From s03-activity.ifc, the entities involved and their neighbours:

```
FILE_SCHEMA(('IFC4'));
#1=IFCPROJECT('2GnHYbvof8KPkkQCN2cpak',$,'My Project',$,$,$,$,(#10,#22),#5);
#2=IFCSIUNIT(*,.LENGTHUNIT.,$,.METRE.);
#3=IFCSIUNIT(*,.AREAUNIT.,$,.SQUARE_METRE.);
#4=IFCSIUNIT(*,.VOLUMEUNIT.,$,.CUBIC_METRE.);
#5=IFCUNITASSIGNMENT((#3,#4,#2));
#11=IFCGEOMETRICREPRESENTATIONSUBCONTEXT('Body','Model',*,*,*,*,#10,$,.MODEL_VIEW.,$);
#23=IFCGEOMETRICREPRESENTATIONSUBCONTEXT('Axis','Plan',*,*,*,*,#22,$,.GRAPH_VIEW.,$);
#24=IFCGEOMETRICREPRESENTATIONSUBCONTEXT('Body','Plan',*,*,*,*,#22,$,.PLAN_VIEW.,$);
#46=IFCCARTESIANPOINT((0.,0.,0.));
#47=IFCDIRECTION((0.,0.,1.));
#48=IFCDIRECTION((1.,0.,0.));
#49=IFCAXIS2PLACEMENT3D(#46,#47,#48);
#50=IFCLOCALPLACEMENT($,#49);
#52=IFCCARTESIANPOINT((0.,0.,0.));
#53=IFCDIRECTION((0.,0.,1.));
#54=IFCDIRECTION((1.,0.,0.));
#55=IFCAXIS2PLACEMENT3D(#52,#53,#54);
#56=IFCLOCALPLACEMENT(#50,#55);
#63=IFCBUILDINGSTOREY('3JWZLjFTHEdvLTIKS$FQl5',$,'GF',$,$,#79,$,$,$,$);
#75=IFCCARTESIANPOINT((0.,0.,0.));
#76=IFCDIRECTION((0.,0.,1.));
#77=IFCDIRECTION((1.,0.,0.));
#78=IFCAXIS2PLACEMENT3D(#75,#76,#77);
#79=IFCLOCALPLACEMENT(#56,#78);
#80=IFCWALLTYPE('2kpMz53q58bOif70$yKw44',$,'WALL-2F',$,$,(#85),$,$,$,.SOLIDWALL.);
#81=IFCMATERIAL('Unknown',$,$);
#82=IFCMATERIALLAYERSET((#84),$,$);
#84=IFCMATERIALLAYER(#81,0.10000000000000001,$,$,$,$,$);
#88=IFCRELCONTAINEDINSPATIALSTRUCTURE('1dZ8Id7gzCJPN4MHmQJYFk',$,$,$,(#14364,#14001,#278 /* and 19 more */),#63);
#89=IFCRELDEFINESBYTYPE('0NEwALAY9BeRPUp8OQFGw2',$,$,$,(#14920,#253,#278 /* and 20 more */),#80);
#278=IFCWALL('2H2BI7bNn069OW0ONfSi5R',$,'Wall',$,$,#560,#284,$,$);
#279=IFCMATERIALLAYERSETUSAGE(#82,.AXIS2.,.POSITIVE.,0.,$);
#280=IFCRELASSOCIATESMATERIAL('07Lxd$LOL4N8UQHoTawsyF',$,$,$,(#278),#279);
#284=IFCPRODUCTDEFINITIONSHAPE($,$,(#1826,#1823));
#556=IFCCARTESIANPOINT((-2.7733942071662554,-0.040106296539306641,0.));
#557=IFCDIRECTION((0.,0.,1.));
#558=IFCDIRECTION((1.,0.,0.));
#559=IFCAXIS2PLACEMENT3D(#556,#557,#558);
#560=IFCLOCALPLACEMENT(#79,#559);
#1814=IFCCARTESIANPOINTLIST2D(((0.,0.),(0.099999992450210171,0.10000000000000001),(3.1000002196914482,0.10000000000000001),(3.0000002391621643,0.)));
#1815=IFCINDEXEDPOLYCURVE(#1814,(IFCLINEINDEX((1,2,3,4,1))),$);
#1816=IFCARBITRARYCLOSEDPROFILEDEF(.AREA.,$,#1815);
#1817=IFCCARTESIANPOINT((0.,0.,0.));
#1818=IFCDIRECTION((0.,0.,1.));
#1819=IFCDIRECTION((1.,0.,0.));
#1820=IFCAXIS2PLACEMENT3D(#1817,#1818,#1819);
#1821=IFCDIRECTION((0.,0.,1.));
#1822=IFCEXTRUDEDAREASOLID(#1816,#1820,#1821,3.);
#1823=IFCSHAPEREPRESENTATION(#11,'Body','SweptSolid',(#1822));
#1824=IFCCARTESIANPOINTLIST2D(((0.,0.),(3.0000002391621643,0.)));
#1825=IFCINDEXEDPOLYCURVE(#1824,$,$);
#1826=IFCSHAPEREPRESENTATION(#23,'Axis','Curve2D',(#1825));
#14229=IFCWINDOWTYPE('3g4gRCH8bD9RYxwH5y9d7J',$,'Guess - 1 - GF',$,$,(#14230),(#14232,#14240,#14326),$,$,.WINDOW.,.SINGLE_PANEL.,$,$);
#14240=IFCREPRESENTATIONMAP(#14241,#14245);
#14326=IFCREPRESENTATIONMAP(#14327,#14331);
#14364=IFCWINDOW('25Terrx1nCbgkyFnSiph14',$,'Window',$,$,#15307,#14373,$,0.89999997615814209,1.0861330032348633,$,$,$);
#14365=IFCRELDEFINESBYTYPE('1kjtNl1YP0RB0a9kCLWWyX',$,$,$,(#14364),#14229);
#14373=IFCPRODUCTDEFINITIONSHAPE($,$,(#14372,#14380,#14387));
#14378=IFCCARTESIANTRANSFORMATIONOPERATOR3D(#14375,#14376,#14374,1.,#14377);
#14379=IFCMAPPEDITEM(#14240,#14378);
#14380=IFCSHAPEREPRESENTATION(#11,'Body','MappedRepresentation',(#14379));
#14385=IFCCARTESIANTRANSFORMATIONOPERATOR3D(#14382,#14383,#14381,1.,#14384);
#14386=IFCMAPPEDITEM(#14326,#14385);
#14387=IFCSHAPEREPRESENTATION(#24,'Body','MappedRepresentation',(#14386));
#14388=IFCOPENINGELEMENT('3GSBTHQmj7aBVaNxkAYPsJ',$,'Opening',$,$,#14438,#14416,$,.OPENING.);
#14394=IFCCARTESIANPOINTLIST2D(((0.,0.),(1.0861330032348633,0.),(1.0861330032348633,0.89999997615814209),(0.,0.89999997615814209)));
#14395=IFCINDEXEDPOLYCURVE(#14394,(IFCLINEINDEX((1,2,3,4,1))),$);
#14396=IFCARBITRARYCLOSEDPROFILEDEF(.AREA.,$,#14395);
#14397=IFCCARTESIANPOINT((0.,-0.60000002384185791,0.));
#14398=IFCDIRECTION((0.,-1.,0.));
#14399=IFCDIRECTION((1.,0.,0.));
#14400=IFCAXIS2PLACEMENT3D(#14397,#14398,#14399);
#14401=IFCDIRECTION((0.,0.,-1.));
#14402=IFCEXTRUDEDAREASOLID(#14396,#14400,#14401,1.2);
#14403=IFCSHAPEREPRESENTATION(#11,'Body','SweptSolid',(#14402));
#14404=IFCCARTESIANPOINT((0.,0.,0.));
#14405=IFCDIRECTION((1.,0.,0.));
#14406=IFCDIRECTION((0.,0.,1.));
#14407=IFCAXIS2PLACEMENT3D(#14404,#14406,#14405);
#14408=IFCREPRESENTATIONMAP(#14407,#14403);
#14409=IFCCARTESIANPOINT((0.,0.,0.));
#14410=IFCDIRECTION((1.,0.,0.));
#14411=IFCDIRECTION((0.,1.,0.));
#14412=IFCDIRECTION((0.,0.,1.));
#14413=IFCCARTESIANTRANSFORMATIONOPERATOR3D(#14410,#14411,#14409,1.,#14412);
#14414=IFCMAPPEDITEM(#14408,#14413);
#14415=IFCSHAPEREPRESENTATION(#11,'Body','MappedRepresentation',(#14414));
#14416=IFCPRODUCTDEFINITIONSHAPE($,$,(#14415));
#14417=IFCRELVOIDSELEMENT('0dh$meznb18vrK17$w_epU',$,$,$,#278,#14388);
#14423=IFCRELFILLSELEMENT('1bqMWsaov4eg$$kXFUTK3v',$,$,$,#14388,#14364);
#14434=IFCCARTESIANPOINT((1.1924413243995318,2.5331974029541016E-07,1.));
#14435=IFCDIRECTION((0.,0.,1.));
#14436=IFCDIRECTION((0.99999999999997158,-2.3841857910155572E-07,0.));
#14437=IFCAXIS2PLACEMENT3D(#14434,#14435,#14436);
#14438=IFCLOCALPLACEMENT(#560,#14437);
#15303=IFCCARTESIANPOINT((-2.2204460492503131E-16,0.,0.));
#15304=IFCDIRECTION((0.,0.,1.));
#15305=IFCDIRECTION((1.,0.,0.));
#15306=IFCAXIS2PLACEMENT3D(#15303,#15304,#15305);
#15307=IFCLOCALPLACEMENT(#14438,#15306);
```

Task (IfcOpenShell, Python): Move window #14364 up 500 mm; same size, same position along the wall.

```python
import numpy as np
import ifcopenshell
import ifcopenshell.api.geometry
import ifcopenshell.util.placement
import ifcopenshell.util.unit

model = ifcopenshell.open("s03-activity.ifc")
unit_scale = ifcopenshell.util.unit.calculate_unit_scale(model)

window = model.by_guid("25Terrx1nCbgkyFnSiph14")
opening = window.FillsVoids[0].RelatingOpeningElement
dz = 0.5 / unit_scale

shift = np.array([0.0, 0.0, dz])
# The window is placed relative to its opening, so it follows when the opening moves.
matrix = ifcopenshell.util.placement.get_local_placement(opening.ObjectPlacement)
matrix[:3, 3] += shift
ifcopenshell.api.geometry.edit_object_placement(
    model, product=opening, matrix=matrix, is_si=False, should_transform_children=True
)

print(f"moved by {dz * unit_scale:+.3f} m")

model.write("s03-activity_v2.ifc")
```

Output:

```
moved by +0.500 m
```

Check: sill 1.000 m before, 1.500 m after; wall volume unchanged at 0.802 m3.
